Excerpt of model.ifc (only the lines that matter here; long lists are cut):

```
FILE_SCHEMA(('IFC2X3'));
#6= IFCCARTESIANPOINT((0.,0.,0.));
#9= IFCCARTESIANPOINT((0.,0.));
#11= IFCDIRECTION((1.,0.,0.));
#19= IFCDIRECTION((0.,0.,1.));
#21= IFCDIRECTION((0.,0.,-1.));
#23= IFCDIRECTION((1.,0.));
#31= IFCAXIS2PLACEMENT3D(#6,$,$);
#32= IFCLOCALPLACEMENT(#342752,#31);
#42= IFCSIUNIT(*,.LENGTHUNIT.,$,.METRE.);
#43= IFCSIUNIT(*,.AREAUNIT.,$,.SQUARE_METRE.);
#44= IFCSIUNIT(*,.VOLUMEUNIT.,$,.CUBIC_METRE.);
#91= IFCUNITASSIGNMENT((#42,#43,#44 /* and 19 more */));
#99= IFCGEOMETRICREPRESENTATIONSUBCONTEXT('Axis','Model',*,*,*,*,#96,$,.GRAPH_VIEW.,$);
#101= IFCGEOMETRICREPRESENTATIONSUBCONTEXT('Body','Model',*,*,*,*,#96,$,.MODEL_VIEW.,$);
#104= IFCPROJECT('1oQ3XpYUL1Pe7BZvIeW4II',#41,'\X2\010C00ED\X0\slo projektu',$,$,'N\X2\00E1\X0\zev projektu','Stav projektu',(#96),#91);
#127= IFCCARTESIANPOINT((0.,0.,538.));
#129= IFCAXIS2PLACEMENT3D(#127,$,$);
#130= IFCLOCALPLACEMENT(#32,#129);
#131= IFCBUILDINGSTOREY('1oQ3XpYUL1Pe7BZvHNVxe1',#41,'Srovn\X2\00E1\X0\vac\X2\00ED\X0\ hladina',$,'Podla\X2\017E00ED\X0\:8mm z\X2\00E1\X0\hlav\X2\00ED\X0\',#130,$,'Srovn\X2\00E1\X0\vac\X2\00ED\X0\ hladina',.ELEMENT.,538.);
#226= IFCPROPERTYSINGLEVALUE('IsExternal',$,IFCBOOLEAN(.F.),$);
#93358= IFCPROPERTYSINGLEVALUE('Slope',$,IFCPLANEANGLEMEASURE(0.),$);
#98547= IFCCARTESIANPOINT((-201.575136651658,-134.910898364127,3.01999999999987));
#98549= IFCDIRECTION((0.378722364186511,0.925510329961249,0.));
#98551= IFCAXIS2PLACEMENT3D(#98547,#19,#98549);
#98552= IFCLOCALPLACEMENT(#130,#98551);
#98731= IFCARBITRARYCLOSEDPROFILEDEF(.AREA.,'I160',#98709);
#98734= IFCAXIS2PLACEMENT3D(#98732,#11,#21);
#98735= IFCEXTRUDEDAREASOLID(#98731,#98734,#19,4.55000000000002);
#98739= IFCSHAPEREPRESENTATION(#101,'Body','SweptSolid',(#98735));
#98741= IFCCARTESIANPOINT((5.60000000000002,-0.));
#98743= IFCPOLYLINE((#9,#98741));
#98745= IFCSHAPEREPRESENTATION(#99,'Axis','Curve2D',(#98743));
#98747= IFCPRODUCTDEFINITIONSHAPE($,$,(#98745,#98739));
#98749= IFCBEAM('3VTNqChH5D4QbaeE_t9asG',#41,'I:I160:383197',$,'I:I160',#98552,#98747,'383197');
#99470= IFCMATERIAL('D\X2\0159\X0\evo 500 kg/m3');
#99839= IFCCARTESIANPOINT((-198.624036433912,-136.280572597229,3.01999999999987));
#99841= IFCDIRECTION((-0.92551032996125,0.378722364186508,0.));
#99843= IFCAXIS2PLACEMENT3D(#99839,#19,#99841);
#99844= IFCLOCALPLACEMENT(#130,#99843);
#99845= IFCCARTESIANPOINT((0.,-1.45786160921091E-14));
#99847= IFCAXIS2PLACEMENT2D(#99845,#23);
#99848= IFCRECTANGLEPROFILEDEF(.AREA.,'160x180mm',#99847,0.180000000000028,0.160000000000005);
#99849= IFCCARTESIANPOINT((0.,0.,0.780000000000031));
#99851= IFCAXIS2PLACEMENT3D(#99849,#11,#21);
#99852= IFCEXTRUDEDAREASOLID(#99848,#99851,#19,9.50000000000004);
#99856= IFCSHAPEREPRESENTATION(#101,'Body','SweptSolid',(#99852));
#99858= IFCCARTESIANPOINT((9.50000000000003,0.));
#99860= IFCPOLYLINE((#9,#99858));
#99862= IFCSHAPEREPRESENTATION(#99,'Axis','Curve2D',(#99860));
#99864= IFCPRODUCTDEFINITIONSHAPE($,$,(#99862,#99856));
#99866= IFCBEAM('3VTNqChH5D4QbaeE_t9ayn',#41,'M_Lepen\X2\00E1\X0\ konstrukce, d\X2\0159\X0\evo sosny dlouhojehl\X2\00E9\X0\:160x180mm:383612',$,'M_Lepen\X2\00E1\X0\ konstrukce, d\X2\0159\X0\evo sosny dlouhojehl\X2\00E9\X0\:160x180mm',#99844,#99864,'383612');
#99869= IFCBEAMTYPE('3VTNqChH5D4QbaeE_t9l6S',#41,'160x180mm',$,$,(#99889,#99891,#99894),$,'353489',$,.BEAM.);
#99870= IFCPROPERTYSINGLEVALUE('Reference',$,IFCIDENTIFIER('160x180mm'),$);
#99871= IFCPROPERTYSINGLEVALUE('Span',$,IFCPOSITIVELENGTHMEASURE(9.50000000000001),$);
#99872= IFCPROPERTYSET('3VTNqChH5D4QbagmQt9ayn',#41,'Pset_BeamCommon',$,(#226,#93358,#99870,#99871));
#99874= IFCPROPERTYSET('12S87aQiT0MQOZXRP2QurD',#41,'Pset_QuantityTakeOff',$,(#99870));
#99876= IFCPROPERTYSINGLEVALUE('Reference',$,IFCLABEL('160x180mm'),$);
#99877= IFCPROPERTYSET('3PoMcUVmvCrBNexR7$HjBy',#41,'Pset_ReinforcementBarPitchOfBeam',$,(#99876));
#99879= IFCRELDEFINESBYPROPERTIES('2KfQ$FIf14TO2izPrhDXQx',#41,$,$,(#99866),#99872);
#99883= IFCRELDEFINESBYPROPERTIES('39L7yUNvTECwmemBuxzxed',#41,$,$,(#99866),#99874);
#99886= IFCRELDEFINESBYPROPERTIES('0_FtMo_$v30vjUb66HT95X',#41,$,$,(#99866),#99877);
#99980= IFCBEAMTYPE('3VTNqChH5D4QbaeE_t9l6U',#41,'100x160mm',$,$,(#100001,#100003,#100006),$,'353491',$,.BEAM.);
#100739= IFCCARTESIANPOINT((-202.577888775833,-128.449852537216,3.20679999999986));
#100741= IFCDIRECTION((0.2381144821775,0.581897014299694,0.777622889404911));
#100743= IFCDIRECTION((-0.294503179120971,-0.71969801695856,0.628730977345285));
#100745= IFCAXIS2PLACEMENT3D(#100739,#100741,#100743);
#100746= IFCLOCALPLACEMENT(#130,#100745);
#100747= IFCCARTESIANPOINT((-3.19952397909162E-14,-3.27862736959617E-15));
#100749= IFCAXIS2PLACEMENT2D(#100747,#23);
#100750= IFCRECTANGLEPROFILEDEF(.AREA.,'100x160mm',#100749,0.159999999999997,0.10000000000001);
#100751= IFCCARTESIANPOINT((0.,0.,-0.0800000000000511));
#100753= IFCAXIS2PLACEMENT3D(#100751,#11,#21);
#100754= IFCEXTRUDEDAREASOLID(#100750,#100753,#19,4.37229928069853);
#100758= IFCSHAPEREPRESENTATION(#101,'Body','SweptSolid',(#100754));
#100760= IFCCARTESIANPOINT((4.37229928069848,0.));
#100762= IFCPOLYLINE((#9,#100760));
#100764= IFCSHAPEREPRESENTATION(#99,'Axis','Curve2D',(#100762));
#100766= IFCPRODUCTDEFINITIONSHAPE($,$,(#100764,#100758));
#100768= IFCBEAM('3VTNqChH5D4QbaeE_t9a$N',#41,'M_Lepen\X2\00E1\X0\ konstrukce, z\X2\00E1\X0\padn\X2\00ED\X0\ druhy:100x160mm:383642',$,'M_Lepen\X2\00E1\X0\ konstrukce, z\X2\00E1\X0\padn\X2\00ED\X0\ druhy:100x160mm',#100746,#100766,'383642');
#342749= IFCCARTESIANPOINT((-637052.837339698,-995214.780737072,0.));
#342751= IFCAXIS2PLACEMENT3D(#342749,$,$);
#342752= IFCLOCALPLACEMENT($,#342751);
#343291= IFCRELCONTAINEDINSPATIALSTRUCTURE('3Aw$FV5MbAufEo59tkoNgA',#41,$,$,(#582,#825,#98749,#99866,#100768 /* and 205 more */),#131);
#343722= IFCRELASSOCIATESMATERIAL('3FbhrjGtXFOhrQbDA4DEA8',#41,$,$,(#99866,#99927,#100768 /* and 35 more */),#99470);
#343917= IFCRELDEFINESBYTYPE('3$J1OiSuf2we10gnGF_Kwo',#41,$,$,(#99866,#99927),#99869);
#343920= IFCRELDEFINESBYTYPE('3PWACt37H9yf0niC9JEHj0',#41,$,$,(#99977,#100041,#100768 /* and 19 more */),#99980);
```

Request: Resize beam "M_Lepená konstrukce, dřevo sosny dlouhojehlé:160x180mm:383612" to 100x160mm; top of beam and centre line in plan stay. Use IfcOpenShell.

```python
import ifcopenshell
import ifcopenshell.api.pset
import ifcopenshell.api.type
import ifcopenshell.util.element
import ifcopenshell.util.representation

model = ifcopenshell.open("model.ifc")

member = model.by_guid("3VTNqChH5D4QbaeE_t9ayn")
source = next(p for p in model.by_type("IfcRectangleProfileDef") if p.ProfileName == "100x160mm")

body = ifcopenshell.util.representation.get_representation(member, "Model", "Body")
solid = body.Items[0]
old_profile = solid.SweptArea

# Copy the section's sizes but keep this member's own profile position.
profile = ifcopenshell.util.element.copy(model, source)
# Profiles are centred, so shift by half the change in depth to hold the top.
shift = (old_profile.XDim - profile.XDim) / 2
x, y = old_profile.Position.Location.Coordinates
up = (-1.0, 0.0)  # upwards, in the solid's own plane
location = model.createIfcCartesianPoint((x + up[0] * shift, y + up[1] * shift))
profile.Position = model.createIfcAxis2Placement2D(location, old_profile.Position.RefDirection)
solid.SweptArea = profile
if not model.get_total_inverses(old_profile):
    ifcopenshell.util.element.remove_deep2(model, old_profile)

new_type = model.by_guid("3VTNqChH5D4QbaeE_t9l6U")
ifcopenshell.api.type.assign_type(
    model, related_objects=[member], relating_type=new_type, should_map_representations=False
)
member.Name = member.Name.replace("160x180mm", "100x160mm")
member.ObjectType = "M_Lepená konstrukce, dřevo sosny dlouhojehlé:100x160mm"
pset = model.by_id(ifcopenshell.util.element.get_pset(member, "Pset_BeamCommon", should_inherit=False)["id"])
ifcopenshell.api.pset.edit_pset(model, pset=pset, properties={"Reference": "100x160mm"})
pset = model.by_id(ifcopenshell.util.element.get_pset(member, "Pset_QuantityTakeOff", should_inherit=False)["id"])
ifcopenshell.api.pset.edit_pset(model, pset=pset, properties={"Reference": "100x160mm"})
pset = model.by_id(ifcopenshell.util.element.get_pset(member, "Pset_ReinforcementBarPitchOfBeam", should_inherit=False)["id"])
ifcopenshell.api.pset.edit_pset(model, pset=pset, properties={"Reference": "100x160mm"})

print(solid.SweptArea)

model.write("model-out.ifc")
```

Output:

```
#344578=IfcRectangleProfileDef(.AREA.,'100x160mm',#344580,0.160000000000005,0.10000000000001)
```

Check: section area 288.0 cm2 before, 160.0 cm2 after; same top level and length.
